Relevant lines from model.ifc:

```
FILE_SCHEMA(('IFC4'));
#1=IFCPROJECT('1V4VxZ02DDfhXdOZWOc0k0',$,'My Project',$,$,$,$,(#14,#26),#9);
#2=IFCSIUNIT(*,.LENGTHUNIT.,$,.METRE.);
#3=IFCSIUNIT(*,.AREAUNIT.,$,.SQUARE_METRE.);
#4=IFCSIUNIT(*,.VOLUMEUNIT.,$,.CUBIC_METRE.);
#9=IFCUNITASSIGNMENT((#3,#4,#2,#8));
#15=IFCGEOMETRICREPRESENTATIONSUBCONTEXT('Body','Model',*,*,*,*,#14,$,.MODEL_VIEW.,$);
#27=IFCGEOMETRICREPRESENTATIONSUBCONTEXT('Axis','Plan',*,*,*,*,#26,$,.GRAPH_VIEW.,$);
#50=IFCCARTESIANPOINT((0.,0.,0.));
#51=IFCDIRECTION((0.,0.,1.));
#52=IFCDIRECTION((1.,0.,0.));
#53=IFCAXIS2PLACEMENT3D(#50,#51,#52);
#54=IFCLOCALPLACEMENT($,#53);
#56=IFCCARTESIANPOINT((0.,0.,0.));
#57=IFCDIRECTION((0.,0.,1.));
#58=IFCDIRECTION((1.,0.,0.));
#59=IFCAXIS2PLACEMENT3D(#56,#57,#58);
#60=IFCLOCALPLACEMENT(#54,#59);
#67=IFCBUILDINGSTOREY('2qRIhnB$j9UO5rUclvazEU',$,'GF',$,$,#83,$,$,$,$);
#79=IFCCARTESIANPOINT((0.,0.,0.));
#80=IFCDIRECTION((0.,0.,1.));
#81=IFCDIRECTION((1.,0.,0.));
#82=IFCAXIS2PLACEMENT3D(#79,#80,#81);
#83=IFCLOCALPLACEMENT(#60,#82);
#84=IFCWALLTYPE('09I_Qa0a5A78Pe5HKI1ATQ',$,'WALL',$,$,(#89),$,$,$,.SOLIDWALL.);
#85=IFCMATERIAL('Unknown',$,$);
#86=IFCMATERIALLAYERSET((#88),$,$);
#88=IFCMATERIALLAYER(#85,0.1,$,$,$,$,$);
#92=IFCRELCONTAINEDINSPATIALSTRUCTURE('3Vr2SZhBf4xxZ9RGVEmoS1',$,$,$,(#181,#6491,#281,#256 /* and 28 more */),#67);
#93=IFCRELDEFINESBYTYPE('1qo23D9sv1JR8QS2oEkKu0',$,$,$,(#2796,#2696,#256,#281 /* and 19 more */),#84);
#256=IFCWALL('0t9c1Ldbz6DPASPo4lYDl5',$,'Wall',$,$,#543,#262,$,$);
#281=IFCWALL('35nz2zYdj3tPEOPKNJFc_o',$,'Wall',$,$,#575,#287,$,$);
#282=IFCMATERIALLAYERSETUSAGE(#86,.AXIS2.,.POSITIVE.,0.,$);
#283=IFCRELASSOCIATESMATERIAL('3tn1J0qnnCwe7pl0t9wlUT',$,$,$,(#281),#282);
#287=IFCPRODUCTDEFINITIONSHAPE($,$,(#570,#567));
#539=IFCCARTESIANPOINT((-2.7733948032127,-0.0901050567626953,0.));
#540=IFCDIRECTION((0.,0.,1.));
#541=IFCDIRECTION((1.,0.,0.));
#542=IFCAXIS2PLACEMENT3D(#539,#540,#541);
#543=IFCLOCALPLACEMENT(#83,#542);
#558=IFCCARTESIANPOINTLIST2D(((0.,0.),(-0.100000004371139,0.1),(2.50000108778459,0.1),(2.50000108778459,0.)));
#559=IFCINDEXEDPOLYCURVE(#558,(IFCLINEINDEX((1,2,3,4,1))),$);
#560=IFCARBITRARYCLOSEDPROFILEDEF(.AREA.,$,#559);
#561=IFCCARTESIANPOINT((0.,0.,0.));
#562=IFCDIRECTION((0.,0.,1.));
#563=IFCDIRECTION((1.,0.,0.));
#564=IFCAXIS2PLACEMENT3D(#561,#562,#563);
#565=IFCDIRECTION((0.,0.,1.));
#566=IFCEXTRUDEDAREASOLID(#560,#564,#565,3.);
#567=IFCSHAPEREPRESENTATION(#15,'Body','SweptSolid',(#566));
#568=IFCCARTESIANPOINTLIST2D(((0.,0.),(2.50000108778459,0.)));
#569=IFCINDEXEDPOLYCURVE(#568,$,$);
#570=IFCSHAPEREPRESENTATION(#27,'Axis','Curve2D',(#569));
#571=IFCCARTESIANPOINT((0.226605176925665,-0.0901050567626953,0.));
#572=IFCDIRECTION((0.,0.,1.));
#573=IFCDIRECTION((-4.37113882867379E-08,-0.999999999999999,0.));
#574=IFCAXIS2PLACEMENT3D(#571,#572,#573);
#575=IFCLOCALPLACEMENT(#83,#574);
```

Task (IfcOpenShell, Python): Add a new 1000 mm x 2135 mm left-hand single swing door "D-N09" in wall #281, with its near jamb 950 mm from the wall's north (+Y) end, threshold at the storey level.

```python
import numpy as np
import ifcopenshell
import ifcopenshell.api.feature
import ifcopenshell.api.geometry
import ifcopenshell.api.root
import ifcopenshell.api.spatial
import ifcopenshell.geom
import ifcopenshell.util.element
import ifcopenshell.util.placement
import ifcopenshell.util.representation
import ifcopenshell.util.shape
import ifcopenshell.util.unit

model = ifcopenshell.open("model.ifc")
unit_scale = ifcopenshell.util.unit.calculate_unit_scale(model)
settings = ifcopenshell.geom.settings()


def volume(element):
    """Net volume in cubic metres, openings subtracted."""
    shape = ifcopenshell.geom.create_shape(settings, element)
    return ifcopenshell.util.shape.get_volume(shape.geometry)


wall = model.by_id(281)
storey = ifcopenshell.util.element.get_container(wall, ifc_class="IfcBuildingStorey")
context = ifcopenshell.util.representation.get_context(model, "Model", "Body", "MODEL_VIEW")
before = volume(wall)

width, height, from_end, sill = 1, 2.135, 0.95, 0.0  # metres

# The wall runs along its own X axis, and the end named is its -X end.
wall_shape = ifcopenshell.geom.create_shape(settings, wall)
x, y, z = ifcopenshell.util.shape.get_vertices(wall_shape.geometry).T
start = x.min() + from_end
face, thickness = float(y.min()), float(y.max() - y.min())
wall_matrix = ifcopenshell.util.placement.get_local_placement(wall.ObjectPlacement)
level = ifcopenshell.util.placement.get_local_placement(storey.ObjectPlacement)[2, 3]


def in_wall(x, y):
    """Placement at x, y metres in the wall's axes, at sill height."""
    matrix = wall_matrix.copy()
    matrix[:, 3] = wall_matrix @ np.array([x / unit_scale, y / unit_scale, 0.0, 1.0])
    matrix[2, 3] = level + sill / unit_scale
    return matrix


# Opening: a box that overshoots both wall faces by 50 mm.
opening = ifcopenshell.api.root.create_entity(model, ifc_class="IfcOpeningElement", predefined_type="OPENING")
box = ifcopenshell.api.geometry.add_wall_representation(
    model, context=context, length=width, height=height, thickness=thickness + 0.1
)
ifcopenshell.api.geometry.assign_representation(model, product=opening, representation=box)
ifcopenshell.api.geometry.edit_object_placement(model, product=opening, matrix=in_wall(start, face - 0.05), is_si=False)
ifcopenshell.api.feature.add_feature(model, feature=opening, element=wall)

door = ifcopenshell.api.root.create_entity(model, ifc_class="IfcDoor", name="D-N09", predefined_type="DOOR")
door.OverallWidth, door.OverallHeight = width / unit_scale, height / unit_scale
door.OperationType = "SINGLE_SWING_LEFT"
body = ifcopenshell.api.geometry.add_door_representation(
    model,
    context=context,
    overall_width=door.OverallWidth,
    overall_height=door.OverallHeight,
    operation_type="SINGLE_SWING_LEFT",
    lining_properties={"LiningDepth": thickness / unit_scale, "ThresholdDepth": thickness / unit_scale},
)
ifcopenshell.api.geometry.assign_representation(model, product=door, representation=body)
ifcopenshell.api.spatial.assign_container(model, products=[door], relating_structure=storey)
ifcopenshell.api.feature.add_filling(model, opening=opening, element=door)

# The lining spans the wall, so the door starts at the wall face.
ifcopenshell.api.geometry.edit_object_placement(model, product=door, matrix=in_wall(start, face), is_si=False)

after = volume(wall)

print(f"wall volume {before:.3f} -> {after:.3f} m3")

model.write("model_edited.ifc")
```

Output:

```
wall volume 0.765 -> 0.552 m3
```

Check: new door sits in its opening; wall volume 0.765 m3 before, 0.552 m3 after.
